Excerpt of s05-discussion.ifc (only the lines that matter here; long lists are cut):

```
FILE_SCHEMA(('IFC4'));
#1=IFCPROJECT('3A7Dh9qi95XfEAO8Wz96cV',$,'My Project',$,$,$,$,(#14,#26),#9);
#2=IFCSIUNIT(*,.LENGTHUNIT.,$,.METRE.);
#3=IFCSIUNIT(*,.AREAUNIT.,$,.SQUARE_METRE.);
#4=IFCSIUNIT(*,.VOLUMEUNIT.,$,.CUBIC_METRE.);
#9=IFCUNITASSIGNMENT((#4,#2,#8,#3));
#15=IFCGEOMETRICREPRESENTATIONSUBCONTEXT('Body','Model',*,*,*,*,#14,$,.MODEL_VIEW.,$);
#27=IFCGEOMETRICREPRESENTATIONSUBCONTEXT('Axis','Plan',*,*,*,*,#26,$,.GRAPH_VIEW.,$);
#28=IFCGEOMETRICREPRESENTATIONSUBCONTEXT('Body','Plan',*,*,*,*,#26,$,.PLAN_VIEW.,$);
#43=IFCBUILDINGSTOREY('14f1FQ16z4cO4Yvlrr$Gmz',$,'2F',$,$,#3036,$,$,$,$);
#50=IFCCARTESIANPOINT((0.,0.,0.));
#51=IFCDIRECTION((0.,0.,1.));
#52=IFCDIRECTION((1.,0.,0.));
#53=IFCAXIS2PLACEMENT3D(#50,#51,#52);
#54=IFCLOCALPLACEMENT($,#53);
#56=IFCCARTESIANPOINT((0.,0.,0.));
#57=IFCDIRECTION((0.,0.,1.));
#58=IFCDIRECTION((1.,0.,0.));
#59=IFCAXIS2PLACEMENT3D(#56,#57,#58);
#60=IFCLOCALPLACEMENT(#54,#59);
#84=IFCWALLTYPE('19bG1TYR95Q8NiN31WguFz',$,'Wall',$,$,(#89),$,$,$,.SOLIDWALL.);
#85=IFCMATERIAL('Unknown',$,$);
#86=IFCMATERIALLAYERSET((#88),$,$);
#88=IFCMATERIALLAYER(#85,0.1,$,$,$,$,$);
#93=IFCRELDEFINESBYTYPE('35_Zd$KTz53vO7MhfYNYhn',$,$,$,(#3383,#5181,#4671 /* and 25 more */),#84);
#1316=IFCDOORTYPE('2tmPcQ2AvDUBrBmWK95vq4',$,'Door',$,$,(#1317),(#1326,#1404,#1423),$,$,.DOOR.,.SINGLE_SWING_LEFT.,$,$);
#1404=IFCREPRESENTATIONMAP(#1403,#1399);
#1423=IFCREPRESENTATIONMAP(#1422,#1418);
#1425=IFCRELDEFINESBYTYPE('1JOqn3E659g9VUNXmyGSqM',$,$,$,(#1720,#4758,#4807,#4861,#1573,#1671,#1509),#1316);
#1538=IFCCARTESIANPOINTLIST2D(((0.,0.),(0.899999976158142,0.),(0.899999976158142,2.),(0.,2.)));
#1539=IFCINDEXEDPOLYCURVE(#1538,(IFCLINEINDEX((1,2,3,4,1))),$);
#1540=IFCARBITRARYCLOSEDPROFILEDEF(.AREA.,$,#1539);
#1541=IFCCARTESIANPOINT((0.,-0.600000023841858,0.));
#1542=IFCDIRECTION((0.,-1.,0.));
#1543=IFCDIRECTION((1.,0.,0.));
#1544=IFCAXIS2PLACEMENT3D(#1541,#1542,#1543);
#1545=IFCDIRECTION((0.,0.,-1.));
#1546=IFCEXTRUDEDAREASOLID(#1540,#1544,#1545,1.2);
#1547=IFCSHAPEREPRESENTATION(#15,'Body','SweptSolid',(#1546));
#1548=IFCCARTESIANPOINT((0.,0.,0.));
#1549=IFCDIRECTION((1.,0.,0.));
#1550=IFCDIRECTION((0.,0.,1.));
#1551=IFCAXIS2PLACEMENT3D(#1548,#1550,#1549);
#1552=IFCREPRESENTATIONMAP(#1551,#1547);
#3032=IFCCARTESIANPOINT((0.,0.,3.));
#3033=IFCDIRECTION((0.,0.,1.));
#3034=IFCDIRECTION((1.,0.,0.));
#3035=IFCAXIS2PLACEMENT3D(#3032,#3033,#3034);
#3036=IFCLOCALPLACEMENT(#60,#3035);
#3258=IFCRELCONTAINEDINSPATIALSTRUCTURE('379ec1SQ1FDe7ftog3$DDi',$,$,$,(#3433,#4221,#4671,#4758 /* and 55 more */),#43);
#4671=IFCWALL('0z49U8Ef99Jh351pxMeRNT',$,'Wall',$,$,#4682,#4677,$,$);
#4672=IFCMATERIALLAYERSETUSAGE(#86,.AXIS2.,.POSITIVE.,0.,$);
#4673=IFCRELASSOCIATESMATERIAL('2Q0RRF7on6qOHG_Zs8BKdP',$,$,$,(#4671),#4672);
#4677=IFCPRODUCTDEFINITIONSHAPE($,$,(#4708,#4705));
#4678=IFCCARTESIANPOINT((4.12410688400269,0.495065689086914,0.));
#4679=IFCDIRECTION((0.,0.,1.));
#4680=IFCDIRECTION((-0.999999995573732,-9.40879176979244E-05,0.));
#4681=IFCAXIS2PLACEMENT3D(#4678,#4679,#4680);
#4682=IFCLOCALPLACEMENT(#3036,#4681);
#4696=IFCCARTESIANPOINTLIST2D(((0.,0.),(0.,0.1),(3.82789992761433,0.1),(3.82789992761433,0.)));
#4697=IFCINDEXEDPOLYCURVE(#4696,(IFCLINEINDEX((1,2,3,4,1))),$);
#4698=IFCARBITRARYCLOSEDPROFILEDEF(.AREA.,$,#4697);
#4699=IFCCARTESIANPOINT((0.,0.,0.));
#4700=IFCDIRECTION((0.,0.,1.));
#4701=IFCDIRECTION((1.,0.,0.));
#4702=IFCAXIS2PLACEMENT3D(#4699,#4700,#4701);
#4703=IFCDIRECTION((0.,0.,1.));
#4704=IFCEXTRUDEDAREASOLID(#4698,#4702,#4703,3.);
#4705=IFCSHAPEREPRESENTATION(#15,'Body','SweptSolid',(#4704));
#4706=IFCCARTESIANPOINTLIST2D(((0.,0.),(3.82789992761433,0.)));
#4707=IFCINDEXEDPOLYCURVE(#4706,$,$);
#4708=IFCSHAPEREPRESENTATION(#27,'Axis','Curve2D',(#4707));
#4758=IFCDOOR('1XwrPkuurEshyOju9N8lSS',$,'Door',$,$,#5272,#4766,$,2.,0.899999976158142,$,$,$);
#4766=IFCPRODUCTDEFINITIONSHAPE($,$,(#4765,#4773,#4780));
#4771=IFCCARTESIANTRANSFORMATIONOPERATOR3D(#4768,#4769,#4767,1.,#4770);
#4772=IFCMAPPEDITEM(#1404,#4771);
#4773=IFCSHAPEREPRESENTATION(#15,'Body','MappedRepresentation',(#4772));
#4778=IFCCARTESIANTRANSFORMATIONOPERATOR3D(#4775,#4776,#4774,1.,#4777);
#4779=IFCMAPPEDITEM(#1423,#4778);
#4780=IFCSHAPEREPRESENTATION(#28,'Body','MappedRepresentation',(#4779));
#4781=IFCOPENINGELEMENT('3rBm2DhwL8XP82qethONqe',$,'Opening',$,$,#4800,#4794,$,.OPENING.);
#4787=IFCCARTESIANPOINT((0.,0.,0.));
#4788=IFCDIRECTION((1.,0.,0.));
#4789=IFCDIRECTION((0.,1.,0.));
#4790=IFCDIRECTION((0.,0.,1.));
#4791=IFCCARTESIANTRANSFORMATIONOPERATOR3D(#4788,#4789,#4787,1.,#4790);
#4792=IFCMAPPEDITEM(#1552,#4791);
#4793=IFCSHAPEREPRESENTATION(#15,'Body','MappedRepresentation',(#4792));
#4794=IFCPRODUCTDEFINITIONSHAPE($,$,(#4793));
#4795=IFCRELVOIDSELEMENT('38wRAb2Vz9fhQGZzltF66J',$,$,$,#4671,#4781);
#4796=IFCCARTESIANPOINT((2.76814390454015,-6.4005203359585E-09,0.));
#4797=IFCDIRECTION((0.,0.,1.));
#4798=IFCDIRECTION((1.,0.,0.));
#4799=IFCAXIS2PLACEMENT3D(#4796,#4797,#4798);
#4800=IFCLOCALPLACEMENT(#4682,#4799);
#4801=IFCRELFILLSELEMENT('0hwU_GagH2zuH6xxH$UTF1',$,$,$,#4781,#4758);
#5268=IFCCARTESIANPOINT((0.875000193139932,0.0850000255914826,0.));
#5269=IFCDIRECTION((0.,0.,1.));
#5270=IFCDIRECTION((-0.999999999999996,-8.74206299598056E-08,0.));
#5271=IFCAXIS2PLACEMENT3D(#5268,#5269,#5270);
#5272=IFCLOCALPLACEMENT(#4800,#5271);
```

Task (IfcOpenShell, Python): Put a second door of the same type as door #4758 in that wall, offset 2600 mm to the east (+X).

```python
import ifcopenshell
import ifcopenshell.api.feature
import ifcopenshell.api.geometry
import ifcopenshell.api.root
import ifcopenshell.geom
import ifcopenshell.util.element
import ifcopenshell.util.placement
import ifcopenshell.util.shape

model = ifcopenshell.open("s05-discussion.ifc")
settings = ifcopenshell.geom.settings()


def volume(element):
    """Net volume in cubic metres, openings subtracted."""
    shape = ifcopenshell.geom.create_shape(settings, element)
    return ifcopenshell.util.shape.get_volume(shape.geometry)


door = model.by_guid("1XwrPkuurEshyOju9N8lSS")
opening = door.FillsVoids[0].RelatingOpeningElement
wall = opening.VoidsElements[0].RelatingBuildingElement
before = volume(wall)
shift = ifcopenshell.util.placement.get_local_placement(wall.ObjectPlacement)[:3, 0] * -2.6

# copy_class copies the void relationship, type, container and properties, but no geometry.
new_opening = ifcopenshell.api.root.copy_class(model, product=opening)
new_opening.Representation = ifcopenshell.util.element.copy_deep(
    model, opening.Representation, exclude=["IfcGeometricRepresentationContext", "IfcRepresentationMap"]
)
new_door = ifcopenshell.api.root.copy_class(model, product=door)
new_door.Representation = ifcopenshell.util.element.copy_deep(
    model, door.Representation, exclude=["IfcGeometricRepresentationContext", "IfcRepresentationMap"]
)
ifcopenshell.api.feature.add_filling(model, opening=new_opening, element=new_door)

for old, new in ((opening, new_opening), (door, new_door)):
    matrix = ifcopenshell.util.placement.get_local_placement(old.ObjectPlacement)
    matrix[:3, 3] += shift
    ifcopenshell.api.geometry.edit_object_placement(model, product=new, matrix=matrix, is_si=False)

after = volume(wall)

print(f"wall volume {before:.3f} -> {after:.3f} m3")

model.write("s05-discussion_v2.ifc")
```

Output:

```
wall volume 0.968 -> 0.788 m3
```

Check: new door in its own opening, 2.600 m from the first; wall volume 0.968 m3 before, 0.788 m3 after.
